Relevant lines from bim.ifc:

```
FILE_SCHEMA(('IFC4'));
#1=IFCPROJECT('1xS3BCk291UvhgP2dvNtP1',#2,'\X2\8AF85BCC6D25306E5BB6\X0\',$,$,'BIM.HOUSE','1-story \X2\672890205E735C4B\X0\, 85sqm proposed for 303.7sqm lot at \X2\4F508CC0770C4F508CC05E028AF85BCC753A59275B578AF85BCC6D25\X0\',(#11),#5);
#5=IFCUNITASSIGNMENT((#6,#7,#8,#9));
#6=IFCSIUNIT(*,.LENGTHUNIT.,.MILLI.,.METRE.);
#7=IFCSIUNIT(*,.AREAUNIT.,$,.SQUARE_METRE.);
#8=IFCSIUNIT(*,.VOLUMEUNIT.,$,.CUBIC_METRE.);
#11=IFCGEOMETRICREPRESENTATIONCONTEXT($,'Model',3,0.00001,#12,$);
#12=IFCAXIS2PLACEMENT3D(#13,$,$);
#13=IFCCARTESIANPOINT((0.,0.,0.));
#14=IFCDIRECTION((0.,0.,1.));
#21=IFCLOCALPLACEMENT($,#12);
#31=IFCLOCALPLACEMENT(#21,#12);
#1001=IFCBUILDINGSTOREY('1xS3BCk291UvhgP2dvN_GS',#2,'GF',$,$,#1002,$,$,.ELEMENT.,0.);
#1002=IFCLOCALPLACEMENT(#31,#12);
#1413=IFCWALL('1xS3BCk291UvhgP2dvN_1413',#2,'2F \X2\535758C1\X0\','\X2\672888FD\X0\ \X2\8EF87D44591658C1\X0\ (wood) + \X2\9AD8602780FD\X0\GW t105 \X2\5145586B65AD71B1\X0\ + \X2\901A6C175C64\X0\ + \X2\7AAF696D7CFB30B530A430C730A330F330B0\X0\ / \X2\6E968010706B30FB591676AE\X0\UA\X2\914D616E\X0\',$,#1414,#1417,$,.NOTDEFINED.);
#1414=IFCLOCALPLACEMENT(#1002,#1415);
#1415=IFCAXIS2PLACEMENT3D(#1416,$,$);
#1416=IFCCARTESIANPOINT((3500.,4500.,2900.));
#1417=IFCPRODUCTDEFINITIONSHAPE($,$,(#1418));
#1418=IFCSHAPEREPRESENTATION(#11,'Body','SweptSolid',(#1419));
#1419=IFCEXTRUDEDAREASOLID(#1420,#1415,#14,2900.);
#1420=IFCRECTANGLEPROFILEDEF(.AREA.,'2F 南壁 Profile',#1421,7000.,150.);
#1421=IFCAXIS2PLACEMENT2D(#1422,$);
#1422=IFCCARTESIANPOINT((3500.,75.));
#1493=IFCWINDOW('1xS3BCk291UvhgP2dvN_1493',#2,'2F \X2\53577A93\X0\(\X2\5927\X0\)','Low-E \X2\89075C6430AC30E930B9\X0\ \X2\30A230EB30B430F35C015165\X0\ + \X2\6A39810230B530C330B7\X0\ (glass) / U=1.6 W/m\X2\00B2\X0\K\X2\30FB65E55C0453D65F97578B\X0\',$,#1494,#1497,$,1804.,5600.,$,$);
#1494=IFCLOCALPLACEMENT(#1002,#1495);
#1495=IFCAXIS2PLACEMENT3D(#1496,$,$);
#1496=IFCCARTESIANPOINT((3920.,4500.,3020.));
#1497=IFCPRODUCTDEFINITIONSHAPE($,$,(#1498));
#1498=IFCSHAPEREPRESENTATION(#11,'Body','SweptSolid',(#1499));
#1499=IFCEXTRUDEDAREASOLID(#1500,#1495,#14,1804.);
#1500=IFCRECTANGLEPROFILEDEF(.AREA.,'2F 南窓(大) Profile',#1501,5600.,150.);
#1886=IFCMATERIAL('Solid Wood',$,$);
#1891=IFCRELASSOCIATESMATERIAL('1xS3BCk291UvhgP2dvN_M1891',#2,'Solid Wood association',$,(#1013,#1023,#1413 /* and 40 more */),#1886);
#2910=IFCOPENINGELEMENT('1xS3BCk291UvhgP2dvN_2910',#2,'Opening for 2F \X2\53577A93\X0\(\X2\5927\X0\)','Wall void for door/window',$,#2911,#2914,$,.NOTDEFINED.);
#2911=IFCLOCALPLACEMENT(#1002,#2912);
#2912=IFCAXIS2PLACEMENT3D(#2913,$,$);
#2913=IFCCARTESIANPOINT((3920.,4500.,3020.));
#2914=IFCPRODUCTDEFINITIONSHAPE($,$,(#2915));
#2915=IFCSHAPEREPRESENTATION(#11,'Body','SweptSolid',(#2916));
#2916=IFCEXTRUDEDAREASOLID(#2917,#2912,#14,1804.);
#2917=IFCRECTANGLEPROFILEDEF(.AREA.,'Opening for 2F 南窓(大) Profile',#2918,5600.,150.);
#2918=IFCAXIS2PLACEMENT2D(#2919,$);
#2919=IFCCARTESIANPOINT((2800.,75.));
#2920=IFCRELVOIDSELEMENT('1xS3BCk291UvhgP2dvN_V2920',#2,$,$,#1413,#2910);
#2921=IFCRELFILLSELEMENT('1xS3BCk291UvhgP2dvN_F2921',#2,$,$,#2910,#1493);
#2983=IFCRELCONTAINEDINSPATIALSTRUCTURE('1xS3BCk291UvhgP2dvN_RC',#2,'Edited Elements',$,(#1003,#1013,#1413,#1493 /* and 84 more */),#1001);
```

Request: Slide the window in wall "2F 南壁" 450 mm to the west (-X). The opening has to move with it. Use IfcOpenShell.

```python
import ifcopenshell
import ifcopenshell.api.geometry
import ifcopenshell.util.placement

model = ifcopenshell.open("bim.ifc")

window = model.by_guid("1xS3BCk291UvhgP2dvN_1493")
opening = window.FillsVoids[0].RelatingOpeningElement
wall = opening.VoidsElements[0].RelatingBuildingElement

wall_matrix = ifcopenshell.util.placement.get_local_placement(wall.ObjectPlacement)
shift = wall_matrix[:3, 0] * -450.0
before = ifcopenshell.util.placement.get_local_placement(window.ObjectPlacement)[:3, 3].copy()

# The window is not placed relative to its opening, so move both.
for product in (opening, window):
    matrix = ifcopenshell.util.placement.get_local_placement(product.ObjectPlacement)
    matrix[:3, 3] += shift
    ifcopenshell.api.geometry.edit_object_placement(model, product=product, matrix=matrix, is_si=False)

after = ifcopenshell.util.placement.get_local_placement(window.ObjectPlacement)[:3, 3]
print("window moved by", (after - before).round(3) + 0.0)

model.write("bim-out.ifc")
```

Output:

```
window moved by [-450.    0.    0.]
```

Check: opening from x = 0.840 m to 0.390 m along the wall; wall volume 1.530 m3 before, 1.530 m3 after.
